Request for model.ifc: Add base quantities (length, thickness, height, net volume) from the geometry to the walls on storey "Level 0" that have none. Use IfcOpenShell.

First a look at what the model holds.

```python
import ifcopenshell
import ifcopenshell.util.element
import ifcopenshell.util.unit

model = ifcopenshell.open("model.ifc")
print(model.schema)
for unit_type in ("LENGTHUNIT", "AREAUNIT", "VOLUMEUNIT"):
    print(unit_type, ifcopenshell.util.unit.calculate_unit_scale(model, unit_type))
storey = next(s for s in model.by_type("IfcBuildingStorey") if s.Name == "Level 0")
walls = [e for e in ifcopenshell.util.element.get_decomposition(storey) if e.is_a("IfcWall")]
for e in sorted(walls, key=lambda e: e.id()):
    print(e.id(), e.is_a(), e.Name, list(ifcopenshell.util.element.get_psets(e, qtos_only=True)), sep=" | ")
```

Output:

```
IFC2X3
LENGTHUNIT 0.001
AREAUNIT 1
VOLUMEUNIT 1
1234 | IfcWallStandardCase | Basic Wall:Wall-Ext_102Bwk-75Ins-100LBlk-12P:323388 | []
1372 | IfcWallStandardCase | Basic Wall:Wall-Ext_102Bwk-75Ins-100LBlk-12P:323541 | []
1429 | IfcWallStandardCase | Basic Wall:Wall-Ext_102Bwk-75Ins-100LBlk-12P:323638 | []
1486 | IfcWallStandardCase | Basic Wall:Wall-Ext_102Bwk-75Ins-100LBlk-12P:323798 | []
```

```python
import ifcopenshell
import ifcopenshell.api.pset
import ifcopenshell.geom
import ifcopenshell.util.element
import ifcopenshell.util.shape
import ifcopenshell.util.unit

model = ifcopenshell.open("model.ifc")
unit_scale = ifcopenshell.util.unit.calculate_unit_scale(model)
volume_scale = ifcopenshell.util.unit.calculate_unit_scale(model, "VOLUMEUNIT")
settings = ifcopenshell.geom.settings()

storey = next(s for s in model.by_type("IfcBuildingStorey") if s.Name == "Level 0")
walls = [e for e in ifcopenshell.util.element.get_decomposition(storey) if e.is_a("IfcWall")]

for e in sorted(walls, key=lambda e: e.id()):
    if ifcopenshell.util.element.get_psets(e, qtos_only=True, should_inherit=False):
        continue
    # Geometry comes back in metres, in the element's own axes.
    shape = ifcopenshell.geom.create_shape(settings, e)
    values = {
        "Length": ifcopenshell.util.shape.get_x(shape.geometry) / unit_scale,
        "Width": ifcopenshell.util.shape.get_y(shape.geometry) / unit_scale,
        "Height": ifcopenshell.util.shape.get_z(shape.geometry) / unit_scale,
        "NetVolume": ifcopenshell.util.shape.get_volume(shape.geometry) / volume_scale,
    }
    qto = ifcopenshell.api.pset.add_qto(model, product=e, name="BaseQuantities")
    ifcopenshell.api.pset.edit_qto(model, qto=qto, properties=values)
    print(e.id(), {k: round(v, 3) for k, v in values.items()})

model.write("model_edited.ifc")
```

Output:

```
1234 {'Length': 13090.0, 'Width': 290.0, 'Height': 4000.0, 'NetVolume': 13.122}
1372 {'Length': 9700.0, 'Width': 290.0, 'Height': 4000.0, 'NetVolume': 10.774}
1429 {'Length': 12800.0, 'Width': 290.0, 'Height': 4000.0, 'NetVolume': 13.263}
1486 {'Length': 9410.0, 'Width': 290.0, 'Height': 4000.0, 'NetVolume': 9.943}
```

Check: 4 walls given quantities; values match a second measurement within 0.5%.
